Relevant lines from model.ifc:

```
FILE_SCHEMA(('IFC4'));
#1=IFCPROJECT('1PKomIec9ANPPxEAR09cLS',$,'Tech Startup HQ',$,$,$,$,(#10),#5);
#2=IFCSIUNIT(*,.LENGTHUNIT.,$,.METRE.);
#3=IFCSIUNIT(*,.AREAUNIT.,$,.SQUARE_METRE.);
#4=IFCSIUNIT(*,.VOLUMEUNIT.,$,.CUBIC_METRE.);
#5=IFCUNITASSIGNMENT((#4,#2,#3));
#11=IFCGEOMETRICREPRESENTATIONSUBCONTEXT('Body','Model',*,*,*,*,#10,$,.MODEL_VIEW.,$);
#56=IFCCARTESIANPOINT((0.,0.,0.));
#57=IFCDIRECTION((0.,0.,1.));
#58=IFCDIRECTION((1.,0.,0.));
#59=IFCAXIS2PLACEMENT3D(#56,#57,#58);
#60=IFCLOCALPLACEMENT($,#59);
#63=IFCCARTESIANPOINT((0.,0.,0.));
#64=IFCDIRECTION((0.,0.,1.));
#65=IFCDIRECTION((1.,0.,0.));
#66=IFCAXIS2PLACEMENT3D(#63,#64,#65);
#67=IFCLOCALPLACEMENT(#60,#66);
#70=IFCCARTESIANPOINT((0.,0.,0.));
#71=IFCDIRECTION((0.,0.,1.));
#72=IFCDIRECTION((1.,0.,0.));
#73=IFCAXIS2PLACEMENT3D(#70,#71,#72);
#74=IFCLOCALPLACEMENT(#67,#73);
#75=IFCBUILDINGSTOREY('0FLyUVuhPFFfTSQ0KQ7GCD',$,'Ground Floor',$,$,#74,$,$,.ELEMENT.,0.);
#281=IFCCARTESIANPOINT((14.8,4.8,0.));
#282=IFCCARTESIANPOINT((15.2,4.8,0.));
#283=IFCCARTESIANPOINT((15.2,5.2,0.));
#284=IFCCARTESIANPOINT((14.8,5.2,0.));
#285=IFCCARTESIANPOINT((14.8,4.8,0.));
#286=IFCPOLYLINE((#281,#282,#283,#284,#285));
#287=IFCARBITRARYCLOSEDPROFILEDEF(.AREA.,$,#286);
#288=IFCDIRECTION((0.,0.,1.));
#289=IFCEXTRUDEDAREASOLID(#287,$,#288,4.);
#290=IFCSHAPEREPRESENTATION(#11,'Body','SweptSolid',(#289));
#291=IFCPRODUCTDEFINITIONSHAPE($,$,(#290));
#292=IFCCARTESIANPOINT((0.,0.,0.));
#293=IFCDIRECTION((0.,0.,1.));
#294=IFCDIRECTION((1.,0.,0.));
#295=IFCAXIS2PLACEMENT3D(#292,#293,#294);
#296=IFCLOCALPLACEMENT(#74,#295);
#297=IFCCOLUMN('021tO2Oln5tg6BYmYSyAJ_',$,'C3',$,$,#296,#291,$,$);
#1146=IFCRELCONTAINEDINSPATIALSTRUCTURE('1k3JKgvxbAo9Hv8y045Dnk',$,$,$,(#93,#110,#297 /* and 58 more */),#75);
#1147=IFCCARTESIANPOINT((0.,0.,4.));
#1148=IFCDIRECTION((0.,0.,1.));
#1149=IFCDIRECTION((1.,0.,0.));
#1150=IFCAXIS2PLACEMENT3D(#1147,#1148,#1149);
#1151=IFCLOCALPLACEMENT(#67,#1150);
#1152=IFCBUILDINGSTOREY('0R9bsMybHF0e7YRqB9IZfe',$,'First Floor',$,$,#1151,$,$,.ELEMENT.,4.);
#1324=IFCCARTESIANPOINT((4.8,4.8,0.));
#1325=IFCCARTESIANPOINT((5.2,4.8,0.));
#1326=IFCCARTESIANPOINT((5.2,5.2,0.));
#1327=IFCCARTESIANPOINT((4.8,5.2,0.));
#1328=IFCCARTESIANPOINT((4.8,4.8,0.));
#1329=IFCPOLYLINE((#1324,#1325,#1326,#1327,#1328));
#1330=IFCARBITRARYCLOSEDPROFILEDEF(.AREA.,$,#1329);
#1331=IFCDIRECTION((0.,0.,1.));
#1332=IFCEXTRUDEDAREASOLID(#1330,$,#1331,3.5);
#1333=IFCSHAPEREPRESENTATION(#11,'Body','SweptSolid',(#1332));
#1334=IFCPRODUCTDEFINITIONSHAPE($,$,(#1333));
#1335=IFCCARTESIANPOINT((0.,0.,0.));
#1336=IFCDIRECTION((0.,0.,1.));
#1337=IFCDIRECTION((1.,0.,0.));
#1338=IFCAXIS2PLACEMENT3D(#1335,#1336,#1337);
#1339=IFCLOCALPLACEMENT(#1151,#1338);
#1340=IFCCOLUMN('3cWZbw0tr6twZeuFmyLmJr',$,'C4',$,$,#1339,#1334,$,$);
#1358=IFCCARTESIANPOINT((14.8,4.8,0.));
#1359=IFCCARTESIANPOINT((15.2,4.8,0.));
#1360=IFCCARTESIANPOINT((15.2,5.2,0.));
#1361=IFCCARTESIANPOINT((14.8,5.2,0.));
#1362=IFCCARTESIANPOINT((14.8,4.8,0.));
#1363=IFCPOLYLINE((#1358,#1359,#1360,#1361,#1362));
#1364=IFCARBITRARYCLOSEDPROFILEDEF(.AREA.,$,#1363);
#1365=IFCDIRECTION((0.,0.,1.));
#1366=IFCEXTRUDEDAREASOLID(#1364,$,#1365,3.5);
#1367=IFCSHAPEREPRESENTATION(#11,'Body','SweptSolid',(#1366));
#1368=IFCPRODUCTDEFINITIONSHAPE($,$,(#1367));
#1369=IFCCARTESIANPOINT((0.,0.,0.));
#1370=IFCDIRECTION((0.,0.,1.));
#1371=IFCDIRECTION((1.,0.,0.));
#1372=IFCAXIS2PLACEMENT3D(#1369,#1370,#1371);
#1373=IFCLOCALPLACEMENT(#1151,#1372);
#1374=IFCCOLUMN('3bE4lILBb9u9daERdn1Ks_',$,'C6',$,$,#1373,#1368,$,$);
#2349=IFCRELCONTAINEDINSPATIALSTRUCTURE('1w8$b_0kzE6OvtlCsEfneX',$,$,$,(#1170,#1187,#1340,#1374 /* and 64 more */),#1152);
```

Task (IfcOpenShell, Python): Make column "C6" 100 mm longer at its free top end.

```python
import ifcopenshell
import ifcopenshell.util.representation

model = ifcopenshell.open("model.ifc")

member = model.by_guid("3bE4lILBb9u9daERdn1Ks_")
change = 0.1

# The extrusion runs towards the end named, so only its depth changes.
body = ifcopenshell.util.representation.get_representation(member, "Model", "Body")
solid = body.Items[0]
old_length = solid.Depth
solid.Depth += change

print(f"length {old_length:g} -> {solid.Depth:g}")

model.write("model_edited.ifc")
```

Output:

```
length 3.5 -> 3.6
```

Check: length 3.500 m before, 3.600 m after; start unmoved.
